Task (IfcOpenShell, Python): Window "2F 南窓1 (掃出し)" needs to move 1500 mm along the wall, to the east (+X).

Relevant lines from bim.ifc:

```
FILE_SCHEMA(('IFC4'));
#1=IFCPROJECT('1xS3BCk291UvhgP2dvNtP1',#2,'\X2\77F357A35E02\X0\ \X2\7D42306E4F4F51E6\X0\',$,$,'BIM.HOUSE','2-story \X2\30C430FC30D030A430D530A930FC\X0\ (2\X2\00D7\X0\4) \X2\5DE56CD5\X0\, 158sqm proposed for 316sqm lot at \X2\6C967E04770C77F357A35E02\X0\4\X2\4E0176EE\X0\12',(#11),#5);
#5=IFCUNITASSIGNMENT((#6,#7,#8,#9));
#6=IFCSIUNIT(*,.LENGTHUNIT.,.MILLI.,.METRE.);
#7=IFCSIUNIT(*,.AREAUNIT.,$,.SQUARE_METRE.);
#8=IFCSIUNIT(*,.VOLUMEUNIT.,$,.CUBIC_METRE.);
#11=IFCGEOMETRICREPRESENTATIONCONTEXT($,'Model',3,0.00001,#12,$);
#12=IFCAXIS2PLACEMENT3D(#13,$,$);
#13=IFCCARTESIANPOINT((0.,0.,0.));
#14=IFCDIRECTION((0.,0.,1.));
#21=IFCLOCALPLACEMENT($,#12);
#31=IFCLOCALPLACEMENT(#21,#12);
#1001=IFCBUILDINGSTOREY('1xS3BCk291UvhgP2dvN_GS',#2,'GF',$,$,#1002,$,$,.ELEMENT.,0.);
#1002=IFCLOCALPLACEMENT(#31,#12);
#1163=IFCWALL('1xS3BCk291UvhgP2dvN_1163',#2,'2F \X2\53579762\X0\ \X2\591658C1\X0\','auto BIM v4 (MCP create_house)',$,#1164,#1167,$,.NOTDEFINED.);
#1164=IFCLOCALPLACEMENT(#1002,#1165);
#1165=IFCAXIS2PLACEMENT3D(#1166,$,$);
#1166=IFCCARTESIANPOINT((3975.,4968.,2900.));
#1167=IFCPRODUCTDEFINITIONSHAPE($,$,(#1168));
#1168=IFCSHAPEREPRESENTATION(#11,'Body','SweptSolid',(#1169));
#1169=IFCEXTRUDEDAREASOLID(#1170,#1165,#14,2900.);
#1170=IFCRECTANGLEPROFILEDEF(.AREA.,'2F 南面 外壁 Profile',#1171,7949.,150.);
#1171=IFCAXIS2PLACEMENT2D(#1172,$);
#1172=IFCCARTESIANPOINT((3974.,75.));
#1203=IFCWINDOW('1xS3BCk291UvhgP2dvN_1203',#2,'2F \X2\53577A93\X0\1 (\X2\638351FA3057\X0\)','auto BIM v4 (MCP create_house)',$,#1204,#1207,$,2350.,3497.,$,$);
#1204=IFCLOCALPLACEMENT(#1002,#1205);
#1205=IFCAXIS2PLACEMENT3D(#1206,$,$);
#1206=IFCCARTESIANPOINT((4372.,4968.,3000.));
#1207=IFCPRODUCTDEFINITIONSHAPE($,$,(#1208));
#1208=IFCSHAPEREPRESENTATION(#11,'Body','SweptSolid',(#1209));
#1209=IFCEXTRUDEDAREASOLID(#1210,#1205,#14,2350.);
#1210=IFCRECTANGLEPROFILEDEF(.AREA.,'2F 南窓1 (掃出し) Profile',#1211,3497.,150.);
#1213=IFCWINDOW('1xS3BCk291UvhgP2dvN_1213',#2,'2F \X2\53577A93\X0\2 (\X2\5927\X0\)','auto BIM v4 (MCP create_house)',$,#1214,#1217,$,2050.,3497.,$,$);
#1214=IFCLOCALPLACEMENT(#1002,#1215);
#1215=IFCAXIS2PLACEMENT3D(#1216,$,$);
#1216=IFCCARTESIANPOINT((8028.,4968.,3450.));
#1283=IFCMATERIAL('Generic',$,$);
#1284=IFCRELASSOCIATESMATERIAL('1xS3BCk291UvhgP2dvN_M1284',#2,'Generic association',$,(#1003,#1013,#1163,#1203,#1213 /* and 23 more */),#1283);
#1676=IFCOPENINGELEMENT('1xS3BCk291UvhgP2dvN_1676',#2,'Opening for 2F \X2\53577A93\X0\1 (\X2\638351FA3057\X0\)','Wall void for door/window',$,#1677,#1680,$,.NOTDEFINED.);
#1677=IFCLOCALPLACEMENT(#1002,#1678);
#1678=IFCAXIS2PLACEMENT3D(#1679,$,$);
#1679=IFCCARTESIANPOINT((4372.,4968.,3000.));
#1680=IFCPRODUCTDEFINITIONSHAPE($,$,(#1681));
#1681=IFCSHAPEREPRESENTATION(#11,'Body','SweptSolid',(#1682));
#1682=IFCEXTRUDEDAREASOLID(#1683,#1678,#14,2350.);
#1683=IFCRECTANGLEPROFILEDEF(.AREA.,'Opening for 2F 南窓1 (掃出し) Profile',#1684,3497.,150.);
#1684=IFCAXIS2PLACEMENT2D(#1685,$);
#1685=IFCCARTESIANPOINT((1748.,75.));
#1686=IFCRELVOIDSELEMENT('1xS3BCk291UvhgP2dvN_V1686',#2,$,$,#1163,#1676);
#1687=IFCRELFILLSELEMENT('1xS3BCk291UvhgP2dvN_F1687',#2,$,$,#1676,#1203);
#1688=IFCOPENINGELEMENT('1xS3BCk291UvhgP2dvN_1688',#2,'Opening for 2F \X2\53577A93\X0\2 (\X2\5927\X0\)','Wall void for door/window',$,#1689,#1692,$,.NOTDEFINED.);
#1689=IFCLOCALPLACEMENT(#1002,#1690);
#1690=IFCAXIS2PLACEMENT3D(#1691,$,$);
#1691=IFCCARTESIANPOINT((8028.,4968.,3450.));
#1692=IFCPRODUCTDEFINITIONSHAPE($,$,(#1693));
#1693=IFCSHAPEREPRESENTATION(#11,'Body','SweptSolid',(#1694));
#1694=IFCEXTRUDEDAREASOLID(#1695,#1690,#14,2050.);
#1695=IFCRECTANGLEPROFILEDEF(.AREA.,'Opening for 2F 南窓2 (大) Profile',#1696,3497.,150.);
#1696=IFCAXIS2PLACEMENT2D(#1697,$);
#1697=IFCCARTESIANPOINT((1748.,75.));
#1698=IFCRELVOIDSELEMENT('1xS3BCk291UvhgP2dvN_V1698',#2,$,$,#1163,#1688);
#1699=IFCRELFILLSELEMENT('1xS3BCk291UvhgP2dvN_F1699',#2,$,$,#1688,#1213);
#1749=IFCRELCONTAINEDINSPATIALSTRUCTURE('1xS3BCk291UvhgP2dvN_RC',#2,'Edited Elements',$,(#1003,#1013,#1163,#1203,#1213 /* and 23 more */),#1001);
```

```python
import ifcopenshell
import ifcopenshell.api.geometry
import ifcopenshell.util.placement
import ifcopenshell.util.unit

model = ifcopenshell.open("bim.ifc")
unit_scale = ifcopenshell.util.unit.calculate_unit_scale(model)

window = model.by_guid("1xS3BCk291UvhgP2dvN_1203")
opening = window.FillsVoids[0].RelatingOpeningElement
wall = opening.VoidsElements[0].RelatingBuildingElement

wall_matrix = ifcopenshell.util.placement.get_local_placement(wall.ObjectPlacement)
shift = wall_matrix[:3, 0] * 1.5 / unit_scale
before = ifcopenshell.util.placement.get_local_placement(window.ObjectPlacement)[:3, 3].copy()

# The window is not placed relative to its opening, so move both.
for product in (opening, window):
    matrix = ifcopenshell.util.placement.get_local_placement(product.ObjectPlacement)
    matrix[:3, 3] += shift
    ifcopenshell.api.geometry.edit_object_placement(model, product=product, matrix=matrix, is_si=False)

after = ifcopenshell.util.placement.get_local_placement(window.ObjectPlacement)[:3, 3]
print("window moved by", (after - before).round(3) + 0.0)

model.write("bim_v2.ifc")
```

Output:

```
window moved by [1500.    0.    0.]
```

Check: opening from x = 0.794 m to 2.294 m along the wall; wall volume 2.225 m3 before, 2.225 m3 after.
